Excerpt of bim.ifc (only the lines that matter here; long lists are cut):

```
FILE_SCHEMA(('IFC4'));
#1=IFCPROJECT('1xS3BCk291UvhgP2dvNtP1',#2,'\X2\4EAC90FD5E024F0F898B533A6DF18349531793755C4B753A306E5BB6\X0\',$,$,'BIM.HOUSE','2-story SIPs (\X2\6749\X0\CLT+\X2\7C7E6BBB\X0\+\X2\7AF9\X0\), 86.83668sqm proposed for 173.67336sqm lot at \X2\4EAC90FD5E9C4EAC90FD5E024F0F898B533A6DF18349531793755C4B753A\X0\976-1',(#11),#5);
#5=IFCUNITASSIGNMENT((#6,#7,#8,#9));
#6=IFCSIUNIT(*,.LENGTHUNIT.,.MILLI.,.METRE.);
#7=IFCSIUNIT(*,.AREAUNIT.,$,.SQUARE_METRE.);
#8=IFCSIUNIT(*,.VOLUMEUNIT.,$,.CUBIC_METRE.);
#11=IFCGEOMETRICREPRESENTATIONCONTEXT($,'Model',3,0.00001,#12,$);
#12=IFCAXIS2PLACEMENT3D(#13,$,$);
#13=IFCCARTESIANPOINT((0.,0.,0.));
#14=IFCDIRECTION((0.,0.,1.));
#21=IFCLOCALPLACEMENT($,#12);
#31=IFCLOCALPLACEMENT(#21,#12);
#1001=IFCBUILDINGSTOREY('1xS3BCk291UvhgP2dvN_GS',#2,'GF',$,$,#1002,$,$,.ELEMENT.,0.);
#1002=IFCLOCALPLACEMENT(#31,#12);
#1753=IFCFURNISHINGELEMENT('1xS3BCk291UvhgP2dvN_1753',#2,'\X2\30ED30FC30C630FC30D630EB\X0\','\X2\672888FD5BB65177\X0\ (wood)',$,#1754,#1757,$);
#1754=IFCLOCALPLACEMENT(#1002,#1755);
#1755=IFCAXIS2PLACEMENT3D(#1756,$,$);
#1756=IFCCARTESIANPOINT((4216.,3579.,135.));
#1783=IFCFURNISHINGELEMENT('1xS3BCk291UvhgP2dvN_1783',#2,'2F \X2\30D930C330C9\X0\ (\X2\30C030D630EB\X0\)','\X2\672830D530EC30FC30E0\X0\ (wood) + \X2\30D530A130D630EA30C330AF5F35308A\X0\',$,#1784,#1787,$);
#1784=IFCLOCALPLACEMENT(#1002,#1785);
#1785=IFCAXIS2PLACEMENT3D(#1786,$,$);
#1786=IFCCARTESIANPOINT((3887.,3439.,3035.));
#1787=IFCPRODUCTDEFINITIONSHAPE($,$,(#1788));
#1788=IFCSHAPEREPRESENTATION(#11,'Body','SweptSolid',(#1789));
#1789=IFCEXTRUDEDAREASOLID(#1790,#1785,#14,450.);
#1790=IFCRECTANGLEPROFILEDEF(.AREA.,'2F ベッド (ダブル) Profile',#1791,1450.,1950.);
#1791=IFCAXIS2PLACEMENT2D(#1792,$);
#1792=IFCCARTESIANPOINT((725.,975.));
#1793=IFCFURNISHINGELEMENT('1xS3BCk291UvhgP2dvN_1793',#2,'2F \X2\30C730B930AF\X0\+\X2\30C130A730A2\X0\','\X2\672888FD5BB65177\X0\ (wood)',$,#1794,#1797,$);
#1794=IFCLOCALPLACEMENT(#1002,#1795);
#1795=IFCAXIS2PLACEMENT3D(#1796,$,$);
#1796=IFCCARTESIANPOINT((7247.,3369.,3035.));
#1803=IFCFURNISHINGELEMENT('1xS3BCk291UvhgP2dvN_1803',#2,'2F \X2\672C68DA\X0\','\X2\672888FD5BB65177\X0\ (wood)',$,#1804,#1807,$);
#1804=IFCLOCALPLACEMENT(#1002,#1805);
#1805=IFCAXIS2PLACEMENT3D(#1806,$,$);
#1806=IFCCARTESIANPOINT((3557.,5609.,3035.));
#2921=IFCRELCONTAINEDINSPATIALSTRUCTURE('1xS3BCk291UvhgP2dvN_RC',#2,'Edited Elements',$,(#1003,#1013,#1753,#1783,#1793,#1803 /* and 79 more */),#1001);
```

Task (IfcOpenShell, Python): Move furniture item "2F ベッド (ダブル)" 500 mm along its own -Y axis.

```python
import ifcopenshell
import ifcopenshell.api.geometry
import ifcopenshell.util.placement

model = ifcopenshell.open("bim.ifc")

item = model.by_guid("1xS3BCk291UvhgP2dvN_1783")
matrix = ifcopenshell.util.placement.get_local_placement(item.ObjectPlacement)
matrix[:3, 3] -= matrix[:3, 1] * 500.0
ifcopenshell.api.geometry.edit_object_placement(model, product=item, matrix=matrix, is_si=False)

print(ifcopenshell.util.placement.get_local_placement(item.ObjectPlacement).round(3) + 0.0)

model.write("bim_v2.ifc")
```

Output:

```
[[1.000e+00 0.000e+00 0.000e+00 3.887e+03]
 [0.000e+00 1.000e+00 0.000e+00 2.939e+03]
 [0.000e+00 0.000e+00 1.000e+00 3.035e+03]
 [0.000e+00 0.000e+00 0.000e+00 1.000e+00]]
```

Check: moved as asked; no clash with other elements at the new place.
